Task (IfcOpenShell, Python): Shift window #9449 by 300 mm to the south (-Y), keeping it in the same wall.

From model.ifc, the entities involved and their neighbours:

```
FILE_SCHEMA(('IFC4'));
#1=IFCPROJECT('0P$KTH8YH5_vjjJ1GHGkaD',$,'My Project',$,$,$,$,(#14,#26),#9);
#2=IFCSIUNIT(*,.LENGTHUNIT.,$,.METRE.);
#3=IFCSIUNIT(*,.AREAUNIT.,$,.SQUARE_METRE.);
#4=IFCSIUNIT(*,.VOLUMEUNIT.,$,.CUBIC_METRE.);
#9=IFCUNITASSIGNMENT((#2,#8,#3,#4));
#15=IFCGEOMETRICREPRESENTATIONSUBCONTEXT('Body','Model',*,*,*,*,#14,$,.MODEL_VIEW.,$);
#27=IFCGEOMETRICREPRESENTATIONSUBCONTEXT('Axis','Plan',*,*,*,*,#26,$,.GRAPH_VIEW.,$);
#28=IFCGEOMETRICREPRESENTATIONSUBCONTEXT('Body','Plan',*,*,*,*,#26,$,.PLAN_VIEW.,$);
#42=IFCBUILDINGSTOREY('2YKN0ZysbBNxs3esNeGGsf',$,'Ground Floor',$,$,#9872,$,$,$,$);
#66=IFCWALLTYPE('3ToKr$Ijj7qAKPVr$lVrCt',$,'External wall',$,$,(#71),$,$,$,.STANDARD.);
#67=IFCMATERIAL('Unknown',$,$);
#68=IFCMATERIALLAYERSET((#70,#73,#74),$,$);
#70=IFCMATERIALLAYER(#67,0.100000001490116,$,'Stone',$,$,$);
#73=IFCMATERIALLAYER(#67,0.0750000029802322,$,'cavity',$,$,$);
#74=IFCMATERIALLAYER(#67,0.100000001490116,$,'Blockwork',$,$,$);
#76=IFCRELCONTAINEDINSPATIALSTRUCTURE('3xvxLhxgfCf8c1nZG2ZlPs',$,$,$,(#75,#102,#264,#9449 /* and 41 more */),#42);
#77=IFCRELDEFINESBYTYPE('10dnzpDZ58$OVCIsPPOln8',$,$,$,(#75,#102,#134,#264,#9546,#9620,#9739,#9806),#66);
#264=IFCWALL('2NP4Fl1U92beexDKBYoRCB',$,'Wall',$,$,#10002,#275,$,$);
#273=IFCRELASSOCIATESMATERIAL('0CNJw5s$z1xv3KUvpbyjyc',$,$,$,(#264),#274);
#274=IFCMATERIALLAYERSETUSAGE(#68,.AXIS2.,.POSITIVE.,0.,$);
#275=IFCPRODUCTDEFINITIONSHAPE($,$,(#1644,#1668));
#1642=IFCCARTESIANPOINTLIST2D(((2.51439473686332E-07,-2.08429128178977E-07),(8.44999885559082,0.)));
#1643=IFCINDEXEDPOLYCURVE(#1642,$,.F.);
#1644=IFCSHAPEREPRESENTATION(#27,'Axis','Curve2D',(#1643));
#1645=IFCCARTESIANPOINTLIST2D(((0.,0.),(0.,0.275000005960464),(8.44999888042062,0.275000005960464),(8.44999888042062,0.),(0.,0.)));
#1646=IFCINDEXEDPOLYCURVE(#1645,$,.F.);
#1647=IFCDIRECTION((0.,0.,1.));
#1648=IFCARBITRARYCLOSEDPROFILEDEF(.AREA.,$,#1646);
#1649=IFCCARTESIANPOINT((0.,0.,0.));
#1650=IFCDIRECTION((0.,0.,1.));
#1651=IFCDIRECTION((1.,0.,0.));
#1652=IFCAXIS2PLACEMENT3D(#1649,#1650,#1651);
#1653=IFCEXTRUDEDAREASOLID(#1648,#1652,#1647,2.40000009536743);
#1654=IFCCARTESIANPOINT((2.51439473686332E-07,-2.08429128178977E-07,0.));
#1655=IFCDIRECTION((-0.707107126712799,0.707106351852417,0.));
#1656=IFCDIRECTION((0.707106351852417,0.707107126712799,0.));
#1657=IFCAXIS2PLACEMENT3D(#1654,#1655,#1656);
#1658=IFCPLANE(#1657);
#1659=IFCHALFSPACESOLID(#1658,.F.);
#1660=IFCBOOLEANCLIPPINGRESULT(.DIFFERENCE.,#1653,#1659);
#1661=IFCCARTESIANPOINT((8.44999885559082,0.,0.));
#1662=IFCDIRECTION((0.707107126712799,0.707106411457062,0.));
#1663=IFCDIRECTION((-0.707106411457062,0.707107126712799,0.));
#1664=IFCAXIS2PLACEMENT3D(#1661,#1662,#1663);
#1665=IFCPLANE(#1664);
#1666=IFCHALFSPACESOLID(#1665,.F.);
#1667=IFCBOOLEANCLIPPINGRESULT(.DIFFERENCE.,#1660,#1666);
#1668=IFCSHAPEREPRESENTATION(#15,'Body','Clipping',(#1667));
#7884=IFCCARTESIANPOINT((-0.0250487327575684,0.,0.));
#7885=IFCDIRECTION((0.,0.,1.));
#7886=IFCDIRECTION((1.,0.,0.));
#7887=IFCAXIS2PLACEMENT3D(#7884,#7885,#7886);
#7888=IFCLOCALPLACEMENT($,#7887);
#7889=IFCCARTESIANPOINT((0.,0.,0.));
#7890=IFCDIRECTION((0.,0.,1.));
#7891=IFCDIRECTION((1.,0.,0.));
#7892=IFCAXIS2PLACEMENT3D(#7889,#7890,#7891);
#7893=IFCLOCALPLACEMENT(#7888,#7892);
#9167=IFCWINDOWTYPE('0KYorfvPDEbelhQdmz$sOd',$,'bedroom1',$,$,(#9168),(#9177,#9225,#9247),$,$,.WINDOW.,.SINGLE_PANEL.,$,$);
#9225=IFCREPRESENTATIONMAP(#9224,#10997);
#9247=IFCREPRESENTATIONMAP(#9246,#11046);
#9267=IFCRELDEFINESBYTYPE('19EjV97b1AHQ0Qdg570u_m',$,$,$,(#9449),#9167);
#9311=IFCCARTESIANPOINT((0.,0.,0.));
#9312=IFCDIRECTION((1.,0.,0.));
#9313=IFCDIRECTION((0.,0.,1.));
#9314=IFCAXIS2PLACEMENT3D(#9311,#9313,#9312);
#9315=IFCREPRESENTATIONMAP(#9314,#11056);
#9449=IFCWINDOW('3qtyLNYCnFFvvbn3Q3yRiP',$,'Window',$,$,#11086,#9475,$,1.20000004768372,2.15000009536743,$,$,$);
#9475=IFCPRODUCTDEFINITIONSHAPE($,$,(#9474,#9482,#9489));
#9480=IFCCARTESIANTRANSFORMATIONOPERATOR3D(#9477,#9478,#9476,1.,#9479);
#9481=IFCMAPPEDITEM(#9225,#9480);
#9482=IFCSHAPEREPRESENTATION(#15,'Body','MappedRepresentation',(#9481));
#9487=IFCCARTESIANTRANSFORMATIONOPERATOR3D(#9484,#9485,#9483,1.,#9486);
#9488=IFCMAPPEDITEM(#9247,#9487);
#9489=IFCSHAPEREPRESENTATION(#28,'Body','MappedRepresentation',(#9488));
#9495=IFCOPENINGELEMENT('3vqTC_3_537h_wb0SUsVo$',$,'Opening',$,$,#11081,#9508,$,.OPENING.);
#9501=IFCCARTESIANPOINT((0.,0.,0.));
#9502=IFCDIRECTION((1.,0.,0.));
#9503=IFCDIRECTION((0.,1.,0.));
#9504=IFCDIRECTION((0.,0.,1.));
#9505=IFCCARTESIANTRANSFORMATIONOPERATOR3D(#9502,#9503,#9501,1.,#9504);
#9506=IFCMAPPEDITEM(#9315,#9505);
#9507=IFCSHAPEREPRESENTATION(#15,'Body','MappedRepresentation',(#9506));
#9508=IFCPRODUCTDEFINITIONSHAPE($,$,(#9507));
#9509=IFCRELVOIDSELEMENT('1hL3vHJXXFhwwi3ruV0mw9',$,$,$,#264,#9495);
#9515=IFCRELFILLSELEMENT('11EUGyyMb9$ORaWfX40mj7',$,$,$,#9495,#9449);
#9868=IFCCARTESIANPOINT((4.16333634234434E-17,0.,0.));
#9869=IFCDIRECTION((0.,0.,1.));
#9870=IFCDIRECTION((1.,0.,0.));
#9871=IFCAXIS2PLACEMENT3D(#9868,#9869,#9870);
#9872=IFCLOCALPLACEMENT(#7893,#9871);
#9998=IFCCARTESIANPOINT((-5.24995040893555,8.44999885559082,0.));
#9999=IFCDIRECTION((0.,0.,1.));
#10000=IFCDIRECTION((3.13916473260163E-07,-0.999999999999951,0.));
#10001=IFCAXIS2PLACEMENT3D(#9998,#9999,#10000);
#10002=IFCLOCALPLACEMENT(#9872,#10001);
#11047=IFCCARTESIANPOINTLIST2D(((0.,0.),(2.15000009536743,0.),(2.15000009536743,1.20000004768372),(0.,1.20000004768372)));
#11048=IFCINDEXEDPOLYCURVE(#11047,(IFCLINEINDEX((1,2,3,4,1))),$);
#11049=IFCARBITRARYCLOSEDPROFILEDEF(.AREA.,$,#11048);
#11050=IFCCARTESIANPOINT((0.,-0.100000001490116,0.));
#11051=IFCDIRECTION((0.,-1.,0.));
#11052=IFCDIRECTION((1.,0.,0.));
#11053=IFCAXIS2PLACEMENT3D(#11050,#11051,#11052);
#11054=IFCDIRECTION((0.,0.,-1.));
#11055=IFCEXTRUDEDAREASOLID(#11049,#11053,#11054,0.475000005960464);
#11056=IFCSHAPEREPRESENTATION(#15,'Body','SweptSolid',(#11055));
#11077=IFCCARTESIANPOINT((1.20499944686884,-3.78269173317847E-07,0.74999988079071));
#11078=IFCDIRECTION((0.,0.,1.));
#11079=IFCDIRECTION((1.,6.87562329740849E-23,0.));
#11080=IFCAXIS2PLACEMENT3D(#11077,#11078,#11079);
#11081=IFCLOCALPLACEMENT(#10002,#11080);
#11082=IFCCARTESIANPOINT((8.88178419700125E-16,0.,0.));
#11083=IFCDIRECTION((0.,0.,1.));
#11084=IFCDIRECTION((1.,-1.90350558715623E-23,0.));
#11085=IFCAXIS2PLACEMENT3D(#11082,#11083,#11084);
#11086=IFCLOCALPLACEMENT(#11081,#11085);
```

```python
import ifcopenshell
import ifcopenshell.api.geometry
import ifcopenshell.util.placement
import ifcopenshell.util.unit

model = ifcopenshell.open("model.ifc")
unit_scale = ifcopenshell.util.unit.calculate_unit_scale(model)

window = model.by_guid("3qtyLNYCnFFvvbn3Q3yRiP")
opening = window.FillsVoids[0].RelatingOpeningElement
wall = opening.VoidsElements[0].RelatingBuildingElement

wall_matrix = ifcopenshell.util.placement.get_local_placement(wall.ObjectPlacement)
shift = wall_matrix[:3, 0] * 0.3 / unit_scale
before = ifcopenshell.util.placement.get_local_placement(window.ObjectPlacement)[:3, 3].copy()

# The window is placed relative to its opening, so it follows when the opening moves.
matrix = ifcopenshell.util.placement.get_local_placement(opening.ObjectPlacement)
matrix[:3, 3] += shift
ifcopenshell.api.geometry.edit_object_placement(
    model, product=opening, matrix=matrix, is_si=False, should_transform_children=True
)

after = ifcopenshell.util.placement.get_local_placement(window.ObjectPlacement)[:3, 3]
print("window moved by", (after - before).round(3) + 0.0)

model.write("model-out.ifc")
```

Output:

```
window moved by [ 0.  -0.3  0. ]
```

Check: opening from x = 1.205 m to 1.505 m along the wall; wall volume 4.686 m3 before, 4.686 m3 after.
